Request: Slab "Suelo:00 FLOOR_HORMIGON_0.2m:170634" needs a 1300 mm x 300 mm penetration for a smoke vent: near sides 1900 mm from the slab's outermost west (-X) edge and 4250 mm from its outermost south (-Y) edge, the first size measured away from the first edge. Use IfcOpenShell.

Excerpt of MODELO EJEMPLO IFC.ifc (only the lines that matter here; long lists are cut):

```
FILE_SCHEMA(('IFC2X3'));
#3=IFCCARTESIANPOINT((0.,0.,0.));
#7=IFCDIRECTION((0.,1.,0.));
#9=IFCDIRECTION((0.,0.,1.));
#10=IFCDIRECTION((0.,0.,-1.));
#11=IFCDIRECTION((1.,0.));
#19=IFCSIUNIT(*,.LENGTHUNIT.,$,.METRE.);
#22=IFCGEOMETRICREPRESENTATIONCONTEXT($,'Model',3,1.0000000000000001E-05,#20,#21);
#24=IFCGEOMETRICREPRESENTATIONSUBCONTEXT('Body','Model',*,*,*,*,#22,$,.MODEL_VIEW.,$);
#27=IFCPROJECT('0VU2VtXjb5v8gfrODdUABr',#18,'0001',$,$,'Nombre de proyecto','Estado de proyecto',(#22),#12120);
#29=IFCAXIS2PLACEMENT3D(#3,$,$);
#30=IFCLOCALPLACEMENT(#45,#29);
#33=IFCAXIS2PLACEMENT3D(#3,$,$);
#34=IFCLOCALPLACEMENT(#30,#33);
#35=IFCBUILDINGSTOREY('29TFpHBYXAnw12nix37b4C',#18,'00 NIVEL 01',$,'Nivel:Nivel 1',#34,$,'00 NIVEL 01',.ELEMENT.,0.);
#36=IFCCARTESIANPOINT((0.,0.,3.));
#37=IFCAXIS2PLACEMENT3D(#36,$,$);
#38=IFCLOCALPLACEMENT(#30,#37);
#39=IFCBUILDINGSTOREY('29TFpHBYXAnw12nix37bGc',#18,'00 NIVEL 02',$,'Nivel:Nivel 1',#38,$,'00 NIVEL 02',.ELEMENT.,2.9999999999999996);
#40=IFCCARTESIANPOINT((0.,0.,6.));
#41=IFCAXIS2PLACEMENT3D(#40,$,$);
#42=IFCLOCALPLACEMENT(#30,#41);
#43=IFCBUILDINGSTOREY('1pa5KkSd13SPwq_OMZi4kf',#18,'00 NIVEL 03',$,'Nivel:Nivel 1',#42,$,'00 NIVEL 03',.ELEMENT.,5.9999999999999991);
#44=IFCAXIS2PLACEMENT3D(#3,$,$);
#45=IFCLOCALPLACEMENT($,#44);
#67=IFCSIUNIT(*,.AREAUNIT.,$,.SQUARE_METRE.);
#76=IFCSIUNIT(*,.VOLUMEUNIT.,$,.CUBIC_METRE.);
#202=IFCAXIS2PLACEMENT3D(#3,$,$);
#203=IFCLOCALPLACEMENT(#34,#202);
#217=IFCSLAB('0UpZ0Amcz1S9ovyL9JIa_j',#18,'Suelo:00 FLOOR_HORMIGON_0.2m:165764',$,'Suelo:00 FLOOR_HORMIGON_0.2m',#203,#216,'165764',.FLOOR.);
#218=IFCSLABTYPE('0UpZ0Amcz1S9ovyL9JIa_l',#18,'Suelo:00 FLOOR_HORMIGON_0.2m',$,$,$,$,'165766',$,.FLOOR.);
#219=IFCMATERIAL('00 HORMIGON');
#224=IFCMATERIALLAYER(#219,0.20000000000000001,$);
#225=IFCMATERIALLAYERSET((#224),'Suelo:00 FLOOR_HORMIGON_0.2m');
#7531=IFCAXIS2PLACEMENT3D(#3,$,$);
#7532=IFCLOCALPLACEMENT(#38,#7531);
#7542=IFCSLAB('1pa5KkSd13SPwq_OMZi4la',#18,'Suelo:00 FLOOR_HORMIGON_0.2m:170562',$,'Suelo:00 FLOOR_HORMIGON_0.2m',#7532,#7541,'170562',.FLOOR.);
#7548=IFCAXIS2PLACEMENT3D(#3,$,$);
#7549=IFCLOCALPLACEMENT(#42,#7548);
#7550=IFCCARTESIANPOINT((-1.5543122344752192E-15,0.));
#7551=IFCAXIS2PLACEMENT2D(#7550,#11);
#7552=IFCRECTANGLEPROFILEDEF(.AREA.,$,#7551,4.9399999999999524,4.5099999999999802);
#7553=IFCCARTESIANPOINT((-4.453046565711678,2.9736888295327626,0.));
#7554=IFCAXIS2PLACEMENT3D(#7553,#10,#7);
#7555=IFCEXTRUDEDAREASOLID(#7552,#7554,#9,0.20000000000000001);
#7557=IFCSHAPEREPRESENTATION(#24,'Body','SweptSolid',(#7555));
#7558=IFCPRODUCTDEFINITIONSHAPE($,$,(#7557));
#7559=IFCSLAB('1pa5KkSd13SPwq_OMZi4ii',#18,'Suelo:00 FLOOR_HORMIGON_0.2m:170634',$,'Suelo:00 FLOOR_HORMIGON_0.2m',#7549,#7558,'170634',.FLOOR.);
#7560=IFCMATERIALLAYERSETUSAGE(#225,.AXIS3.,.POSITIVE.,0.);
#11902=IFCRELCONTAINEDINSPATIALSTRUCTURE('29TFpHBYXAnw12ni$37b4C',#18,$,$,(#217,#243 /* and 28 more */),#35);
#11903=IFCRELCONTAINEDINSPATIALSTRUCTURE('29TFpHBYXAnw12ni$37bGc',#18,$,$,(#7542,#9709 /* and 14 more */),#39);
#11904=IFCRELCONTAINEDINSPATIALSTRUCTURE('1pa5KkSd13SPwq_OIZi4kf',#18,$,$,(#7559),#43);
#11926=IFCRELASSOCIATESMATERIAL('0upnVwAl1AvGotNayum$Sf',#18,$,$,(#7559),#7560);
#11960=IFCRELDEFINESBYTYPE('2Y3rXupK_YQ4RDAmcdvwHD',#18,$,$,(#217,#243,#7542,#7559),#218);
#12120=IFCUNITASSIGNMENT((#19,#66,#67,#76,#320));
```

```python
import numpy as np
import ifcopenshell
import ifcopenshell.api.feature
import ifcopenshell.api.geometry
import ifcopenshell.api.root
import ifcopenshell.geom
import ifcopenshell.util.placement
import ifcopenshell.util.representation
import ifcopenshell.util.shape
import ifcopenshell.util.unit

model = ifcopenshell.open("MODELO EJEMPLO IFC.ifc")
unit_scale = ifcopenshell.util.unit.calculate_unit_scale(model)
settings = ifcopenshell.geom.settings()


def volume(element):
    """Net volume in cubic metres, openings subtracted."""
    shape = ifcopenshell.geom.create_shape(settings, element)
    return ifcopenshell.util.shape.get_volume(shape.geometry)


slab = model.by_guid("1pa5KkSd13SPwq_OMZi4ii")
before = volume(slab)

# Extent in the slab's own axes, in metres. The edges named are its -X and -Y sides.
slab_shape = ifcopenshell.geom.create_shape(settings, slab)
vertices = ifcopenshell.util.shape.get_vertices(slab_shape.geometry)
x_min, y_min, bottom = vertices.min(axis=0)
top = vertices[:, 2].max()

opening = ifcopenshell.api.root.create_entity(model, ifc_class="IfcOpeningElement", name="Smoke vent opening")
context = ifcopenshell.util.representation.get_context(model, "Model", "Body", "MODEL_VIEW")
width, depth = 1.3, 0.3
outline = [(0.0, 0.0), (width, 0.0), (width, depth), (0.0, depth), (0.0, 0.0)]
# Overshoot both faces by 50 mm so the cut is clean.
shape = ifcopenshell.api.geometry.add_slab_representation(
    model, context=context, depth=top - bottom + 0.1, polyline=outline
)
ifcopenshell.api.geometry.assign_representation(model, product=opening, representation=shape)

matrix = ifcopenshell.util.placement.get_local_placement(slab.ObjectPlacement)
matrix[:, 3] = matrix @ np.append(np.array([x_min + 1.9, y_min + 4.25, bottom - 0.05]) / unit_scale, 1.0)
ifcopenshell.api.geometry.edit_object_placement(model, product=opening, matrix=matrix, is_si=False)
ifcopenshell.api.feature.add_feature(model, feature=opening, element=slab)

after = volume(slab)

print(f"slab volume {before:.3f} -> {after:.3f} m3")

model.write("MODELO EJEMPLO IFC_updated.ifc")
```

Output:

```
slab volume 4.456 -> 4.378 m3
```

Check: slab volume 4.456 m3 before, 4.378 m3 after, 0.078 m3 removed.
